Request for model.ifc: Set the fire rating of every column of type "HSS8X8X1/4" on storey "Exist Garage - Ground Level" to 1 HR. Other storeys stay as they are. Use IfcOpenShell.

First a look at what the model holds.

```python
import ifcopenshell
import ifcopenshell.util.element

model = ifcopenshell.open("model.ifc")
print(model.schema)
storey = next(s for s in model.by_type("IfcBuildingStorey") if s.Name == "Exist Garage - Ground Level")
columns = [e for e in ifcopenshell.util.element.get_decomposition(storey) if e.is_a("IfcColumn")]
seen = {}
for e in columns:
    element_type = ifcopenshell.util.element.get_type(e)
    key = (element_type.Name if element_type != e and element_type else None, ifcopenshell.util.element.get_pset(e, "Pset_ColumnCommon", "FireRating"))
    seen[key] = seen.get(key, 0) + 1
for (name, value), count in sorted(seen.items(), key=str):
    print(count, "x", name, "|", value)
```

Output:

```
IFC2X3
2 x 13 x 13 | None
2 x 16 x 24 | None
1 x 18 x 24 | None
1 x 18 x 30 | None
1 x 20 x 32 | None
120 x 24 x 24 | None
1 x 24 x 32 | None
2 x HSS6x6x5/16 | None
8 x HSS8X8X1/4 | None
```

```python
import ifcopenshell
import ifcopenshell.api.pset
import ifcopenshell.util.element

model = ifcopenshell.open("model.ifc")

storey = next(s for s in model.by_type("IfcBuildingStorey") if s.Name == "Exist Garage - Ground Level")
columns = [e for e in ifcopenshell.util.element.get_decomposition(storey) if e.is_a("IfcColumn")]

count = 0
for e in columns:
    element_type = ifcopenshell.util.element.get_type(e)
    if element_type in (None, e) or element_type.Name != "HSS8X8X1/4":
        continue
    # add_pset returns the element's existing set when there is one.
    pset = ifcopenshell.api.pset.add_pset(model, product=e, name="Pset_ColumnCommon")
    ifcopenshell.api.pset.edit_pset(model, pset=pset, properties={"FireRating": "1 HR"})
    count += 1

print(count, "columns updated")

model.write("model_edited.ifc")
```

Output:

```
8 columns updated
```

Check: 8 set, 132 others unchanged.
